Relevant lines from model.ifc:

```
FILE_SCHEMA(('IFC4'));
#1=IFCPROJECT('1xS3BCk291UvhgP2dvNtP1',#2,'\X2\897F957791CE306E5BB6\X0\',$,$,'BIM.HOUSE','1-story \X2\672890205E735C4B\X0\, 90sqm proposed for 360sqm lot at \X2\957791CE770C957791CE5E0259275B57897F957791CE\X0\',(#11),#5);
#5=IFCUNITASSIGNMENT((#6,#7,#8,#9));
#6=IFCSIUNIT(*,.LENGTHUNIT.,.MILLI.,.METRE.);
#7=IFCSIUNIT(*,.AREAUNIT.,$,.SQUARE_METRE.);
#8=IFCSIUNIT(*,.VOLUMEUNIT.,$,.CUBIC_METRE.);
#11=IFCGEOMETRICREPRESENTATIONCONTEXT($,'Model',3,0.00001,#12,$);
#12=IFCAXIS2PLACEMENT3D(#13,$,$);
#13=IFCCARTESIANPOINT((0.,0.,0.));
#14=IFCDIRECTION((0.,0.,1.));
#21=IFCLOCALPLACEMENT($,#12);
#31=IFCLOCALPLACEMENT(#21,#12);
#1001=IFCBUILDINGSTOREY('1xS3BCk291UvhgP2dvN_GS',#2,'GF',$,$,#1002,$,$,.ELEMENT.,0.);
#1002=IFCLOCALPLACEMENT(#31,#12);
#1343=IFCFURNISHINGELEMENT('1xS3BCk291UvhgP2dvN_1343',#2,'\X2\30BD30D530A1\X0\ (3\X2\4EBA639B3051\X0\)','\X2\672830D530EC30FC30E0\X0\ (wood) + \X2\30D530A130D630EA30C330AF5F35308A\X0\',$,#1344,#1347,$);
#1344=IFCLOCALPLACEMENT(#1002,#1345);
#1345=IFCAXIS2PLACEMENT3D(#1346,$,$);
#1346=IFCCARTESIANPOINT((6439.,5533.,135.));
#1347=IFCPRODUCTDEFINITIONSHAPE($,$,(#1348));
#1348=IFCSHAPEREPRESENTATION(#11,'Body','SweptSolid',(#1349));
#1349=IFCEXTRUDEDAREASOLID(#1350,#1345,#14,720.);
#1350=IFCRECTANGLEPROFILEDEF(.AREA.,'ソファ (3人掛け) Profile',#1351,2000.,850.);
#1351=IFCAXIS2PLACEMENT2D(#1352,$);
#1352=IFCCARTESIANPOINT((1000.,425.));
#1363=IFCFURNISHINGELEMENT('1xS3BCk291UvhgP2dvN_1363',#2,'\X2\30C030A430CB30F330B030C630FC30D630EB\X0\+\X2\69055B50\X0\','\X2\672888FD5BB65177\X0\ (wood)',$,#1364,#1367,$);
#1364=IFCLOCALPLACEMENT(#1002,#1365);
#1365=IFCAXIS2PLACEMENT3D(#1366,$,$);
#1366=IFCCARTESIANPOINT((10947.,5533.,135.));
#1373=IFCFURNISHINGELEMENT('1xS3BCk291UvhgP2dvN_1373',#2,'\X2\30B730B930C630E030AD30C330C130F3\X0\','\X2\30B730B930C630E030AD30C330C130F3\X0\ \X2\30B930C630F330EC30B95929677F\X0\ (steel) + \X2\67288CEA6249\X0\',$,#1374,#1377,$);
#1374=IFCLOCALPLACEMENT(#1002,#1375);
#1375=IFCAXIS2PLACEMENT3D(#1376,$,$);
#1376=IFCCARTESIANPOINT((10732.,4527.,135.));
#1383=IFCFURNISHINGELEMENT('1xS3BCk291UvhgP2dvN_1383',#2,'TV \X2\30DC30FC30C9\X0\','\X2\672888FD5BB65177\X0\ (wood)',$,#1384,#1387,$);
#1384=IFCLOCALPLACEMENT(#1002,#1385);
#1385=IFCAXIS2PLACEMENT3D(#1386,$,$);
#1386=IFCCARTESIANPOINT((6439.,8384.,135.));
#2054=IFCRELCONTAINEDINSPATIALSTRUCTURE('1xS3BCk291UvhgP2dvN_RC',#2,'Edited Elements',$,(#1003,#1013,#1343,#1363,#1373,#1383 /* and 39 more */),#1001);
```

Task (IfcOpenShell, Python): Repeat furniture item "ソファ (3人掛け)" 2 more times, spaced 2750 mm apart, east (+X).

```python
import numpy as np
import ifcopenshell
import ifcopenshell.api.geometry
import ifcopenshell.api.root
import ifcopenshell.util.element
import ifcopenshell.util.placement
import ifcopenshell.util.unit

model = ifcopenshell.open("model.ifc")
unit_scale = ifcopenshell.util.unit.calculate_unit_scale(model)


def reuse_history(source, copy):
    """copy_class also copies each property set's owner history, people and application; keep the originals."""
    for rel in copy.IsDefinedBy:
        if rel.is_a("IfcRelDefinesByProperties") and (history := rel.RelatingPropertyDefinition.OwnerHistory):
            rel.RelatingPropertyDefinition.OwnerHistory = source.OwnerHistory
            ifcopenshell.util.element.remove_deep2(model, history)


source = model.by_id(1343)
base = ifcopenshell.util.placement.get_local_placement(source.ObjectPlacement)
step = np.array([1.0, 0.0, 0.0]) * 2.75 / unit_scale

for i in range(1, 3):
    copy = ifcopenshell.api.root.copy_class(model, product=source)
    copy.Representation = ifcopenshell.util.element.copy_deep(
        model, source.Representation, exclude=["IfcGeometricRepresentationContext", "IfcRepresentationMap"]
    )
    reuse_history(source, copy)
    matrix = base.copy()
    matrix[:3, 3] += i * step
    print("added at", matrix[:3, 3].round(3) + 0.0)
    ifcopenshell.api.geometry.edit_object_placement(model, product=copy, matrix=matrix, is_si=False)

model.write("model_updated.ifc")
```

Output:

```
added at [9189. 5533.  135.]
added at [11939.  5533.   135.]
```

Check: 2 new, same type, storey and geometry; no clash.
